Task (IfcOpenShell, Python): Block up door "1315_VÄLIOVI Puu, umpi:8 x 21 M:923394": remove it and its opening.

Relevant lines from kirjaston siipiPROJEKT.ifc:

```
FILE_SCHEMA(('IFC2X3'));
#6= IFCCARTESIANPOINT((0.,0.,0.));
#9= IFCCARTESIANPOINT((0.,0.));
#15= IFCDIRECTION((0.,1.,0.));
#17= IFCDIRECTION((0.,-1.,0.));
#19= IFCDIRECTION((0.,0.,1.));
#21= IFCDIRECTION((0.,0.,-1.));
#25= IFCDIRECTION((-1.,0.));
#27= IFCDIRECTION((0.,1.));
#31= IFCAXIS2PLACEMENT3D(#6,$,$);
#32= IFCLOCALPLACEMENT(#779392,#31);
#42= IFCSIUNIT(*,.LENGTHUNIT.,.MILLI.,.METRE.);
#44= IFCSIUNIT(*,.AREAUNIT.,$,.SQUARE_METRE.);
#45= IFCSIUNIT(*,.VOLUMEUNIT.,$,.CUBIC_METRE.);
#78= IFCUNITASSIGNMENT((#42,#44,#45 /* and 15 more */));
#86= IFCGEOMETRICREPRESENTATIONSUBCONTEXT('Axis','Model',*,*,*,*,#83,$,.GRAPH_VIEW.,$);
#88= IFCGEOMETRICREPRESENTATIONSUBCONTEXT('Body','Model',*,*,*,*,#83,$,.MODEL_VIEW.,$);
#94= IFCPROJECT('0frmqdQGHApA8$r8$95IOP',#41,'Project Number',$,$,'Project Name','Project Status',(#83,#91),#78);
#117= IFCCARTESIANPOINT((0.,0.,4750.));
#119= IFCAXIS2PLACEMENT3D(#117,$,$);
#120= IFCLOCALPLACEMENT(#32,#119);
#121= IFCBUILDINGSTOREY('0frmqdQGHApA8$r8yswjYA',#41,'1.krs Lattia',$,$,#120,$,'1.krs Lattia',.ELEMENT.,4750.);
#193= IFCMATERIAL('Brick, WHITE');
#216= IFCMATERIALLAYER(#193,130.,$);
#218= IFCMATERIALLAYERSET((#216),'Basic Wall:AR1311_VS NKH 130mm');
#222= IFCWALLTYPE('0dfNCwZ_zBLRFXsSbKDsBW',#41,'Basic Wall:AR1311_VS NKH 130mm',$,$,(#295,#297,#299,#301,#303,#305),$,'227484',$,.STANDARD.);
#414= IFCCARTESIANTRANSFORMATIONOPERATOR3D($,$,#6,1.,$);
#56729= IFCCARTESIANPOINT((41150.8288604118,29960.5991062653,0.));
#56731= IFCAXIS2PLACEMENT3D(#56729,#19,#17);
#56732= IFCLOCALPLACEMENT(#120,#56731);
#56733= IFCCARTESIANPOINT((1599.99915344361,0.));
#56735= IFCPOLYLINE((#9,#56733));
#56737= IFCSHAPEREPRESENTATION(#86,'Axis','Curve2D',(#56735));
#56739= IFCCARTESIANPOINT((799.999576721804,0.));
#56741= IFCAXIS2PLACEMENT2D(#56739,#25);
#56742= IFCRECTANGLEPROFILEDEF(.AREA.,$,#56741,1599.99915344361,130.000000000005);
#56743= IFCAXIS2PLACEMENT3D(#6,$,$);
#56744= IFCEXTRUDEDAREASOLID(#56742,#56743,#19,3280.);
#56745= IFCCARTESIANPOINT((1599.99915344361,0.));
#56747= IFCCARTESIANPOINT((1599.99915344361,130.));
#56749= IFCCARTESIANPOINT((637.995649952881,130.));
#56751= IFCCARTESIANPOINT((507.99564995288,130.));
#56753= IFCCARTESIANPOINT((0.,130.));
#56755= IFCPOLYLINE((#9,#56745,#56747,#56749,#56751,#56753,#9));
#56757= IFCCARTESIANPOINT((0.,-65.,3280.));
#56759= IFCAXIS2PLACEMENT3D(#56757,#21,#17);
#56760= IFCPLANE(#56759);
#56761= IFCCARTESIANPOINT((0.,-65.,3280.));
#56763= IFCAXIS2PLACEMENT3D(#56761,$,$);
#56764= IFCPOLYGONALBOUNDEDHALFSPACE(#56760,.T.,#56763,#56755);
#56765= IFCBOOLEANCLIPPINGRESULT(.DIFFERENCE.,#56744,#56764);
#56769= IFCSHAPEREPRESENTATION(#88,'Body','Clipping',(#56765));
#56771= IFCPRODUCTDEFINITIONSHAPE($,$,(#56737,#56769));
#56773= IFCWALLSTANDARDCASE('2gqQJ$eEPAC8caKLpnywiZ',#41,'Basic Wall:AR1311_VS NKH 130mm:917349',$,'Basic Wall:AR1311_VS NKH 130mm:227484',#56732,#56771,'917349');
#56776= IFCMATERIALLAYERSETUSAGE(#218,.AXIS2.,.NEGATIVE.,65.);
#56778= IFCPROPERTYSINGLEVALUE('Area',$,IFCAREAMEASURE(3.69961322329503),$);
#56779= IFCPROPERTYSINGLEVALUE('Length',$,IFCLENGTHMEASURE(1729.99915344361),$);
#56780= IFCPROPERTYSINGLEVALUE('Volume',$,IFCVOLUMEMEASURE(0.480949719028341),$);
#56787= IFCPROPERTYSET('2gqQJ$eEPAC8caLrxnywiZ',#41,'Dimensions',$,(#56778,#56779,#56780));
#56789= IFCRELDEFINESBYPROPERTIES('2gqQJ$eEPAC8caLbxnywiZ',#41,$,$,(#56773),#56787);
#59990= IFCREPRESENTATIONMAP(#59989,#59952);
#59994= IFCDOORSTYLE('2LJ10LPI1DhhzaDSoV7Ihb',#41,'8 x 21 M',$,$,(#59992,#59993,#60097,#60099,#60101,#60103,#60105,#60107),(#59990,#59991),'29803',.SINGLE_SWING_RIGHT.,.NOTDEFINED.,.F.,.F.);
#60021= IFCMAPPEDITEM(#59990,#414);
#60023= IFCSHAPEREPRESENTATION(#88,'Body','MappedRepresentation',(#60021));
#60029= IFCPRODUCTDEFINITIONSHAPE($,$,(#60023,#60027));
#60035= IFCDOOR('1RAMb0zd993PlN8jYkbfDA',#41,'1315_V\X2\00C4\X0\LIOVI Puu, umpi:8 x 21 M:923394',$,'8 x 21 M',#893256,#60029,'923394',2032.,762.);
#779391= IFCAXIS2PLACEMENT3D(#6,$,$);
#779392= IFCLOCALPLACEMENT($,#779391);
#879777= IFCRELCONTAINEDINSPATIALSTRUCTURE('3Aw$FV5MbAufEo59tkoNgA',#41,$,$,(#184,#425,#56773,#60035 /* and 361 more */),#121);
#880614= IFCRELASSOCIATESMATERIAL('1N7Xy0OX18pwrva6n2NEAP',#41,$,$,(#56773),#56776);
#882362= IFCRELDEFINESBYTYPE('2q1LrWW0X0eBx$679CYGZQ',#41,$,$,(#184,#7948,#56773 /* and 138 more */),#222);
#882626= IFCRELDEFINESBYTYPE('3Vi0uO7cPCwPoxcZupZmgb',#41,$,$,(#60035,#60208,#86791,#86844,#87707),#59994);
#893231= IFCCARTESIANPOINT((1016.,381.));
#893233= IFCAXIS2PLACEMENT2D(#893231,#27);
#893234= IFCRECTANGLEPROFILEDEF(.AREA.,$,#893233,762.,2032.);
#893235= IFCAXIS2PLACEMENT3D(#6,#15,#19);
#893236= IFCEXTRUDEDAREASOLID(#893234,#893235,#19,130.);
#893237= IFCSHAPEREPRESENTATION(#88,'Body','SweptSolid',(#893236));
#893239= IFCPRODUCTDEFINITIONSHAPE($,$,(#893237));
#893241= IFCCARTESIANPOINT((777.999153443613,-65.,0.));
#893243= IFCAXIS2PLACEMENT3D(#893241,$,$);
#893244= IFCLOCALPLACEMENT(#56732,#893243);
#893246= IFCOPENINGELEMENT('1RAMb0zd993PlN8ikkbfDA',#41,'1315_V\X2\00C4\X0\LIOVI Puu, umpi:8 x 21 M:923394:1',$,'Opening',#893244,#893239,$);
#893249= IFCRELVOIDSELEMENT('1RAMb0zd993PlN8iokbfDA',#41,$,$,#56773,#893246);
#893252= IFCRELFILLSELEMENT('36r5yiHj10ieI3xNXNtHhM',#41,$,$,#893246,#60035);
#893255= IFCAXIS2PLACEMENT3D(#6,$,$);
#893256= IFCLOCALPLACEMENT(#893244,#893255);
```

```python
import ifcopenshell
import ifcopenshell.api.feature
import ifcopenshell.api.pset
import ifcopenshell.api.root
import ifcopenshell.geom
import ifcopenshell.util.element
import ifcopenshell.util.shape
import ifcopenshell.util.unit

model = ifcopenshell.open("kirjaston siipiPROJEKT.ifc")
area_scale = ifcopenshell.util.unit.calculate_unit_scale(model, "AREAUNIT")
volume_scale = ifcopenshell.util.unit.calculate_unit_scale(model, "VOLUMEUNIT")
settings = ifcopenshell.geom.settings()


def volume(element):
    """Net volume in cubic metres, openings subtracted."""
    shape = ifcopenshell.geom.create_shape(settings, element)
    return ifcopenshell.util.shape.get_volume(shape.geometry)


door = model.by_guid("1RAMb0zd993PlN8jYkbfDA")
opening = door.FillsVoids[0].RelatingOpeningElement
wall = opening.VoidsElements[0].RelatingBuildingElement
before = volume(wall)

ifcopenshell.api.root.remove_product(model, product=door)
ifcopenshell.api.feature.remove_feature(model, feature=opening)

after = volume(wall)
thickness = 0.13  # wall thickness in metres

# Update the wall's stored quantities.
pset = model.by_id(ifcopenshell.util.element.get_pset(wall, "Dimensions", should_inherit=False)["id"])
ifcopenshell.api.pset.edit_pset(model, pset=pset, properties={
    "Area": model.create_entity("IfcAreaMeasure", after / thickness / area_scale),
    "Volume": model.create_entity("IfcVolumeMeasure", after / volume_scale),
})

print(f"wall volume {before:.3f} -> {after:.3f} m3")

model.write("kirjaston siipiPROJEKT_edited.ifc")
```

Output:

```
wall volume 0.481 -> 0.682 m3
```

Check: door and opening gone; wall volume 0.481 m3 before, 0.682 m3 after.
